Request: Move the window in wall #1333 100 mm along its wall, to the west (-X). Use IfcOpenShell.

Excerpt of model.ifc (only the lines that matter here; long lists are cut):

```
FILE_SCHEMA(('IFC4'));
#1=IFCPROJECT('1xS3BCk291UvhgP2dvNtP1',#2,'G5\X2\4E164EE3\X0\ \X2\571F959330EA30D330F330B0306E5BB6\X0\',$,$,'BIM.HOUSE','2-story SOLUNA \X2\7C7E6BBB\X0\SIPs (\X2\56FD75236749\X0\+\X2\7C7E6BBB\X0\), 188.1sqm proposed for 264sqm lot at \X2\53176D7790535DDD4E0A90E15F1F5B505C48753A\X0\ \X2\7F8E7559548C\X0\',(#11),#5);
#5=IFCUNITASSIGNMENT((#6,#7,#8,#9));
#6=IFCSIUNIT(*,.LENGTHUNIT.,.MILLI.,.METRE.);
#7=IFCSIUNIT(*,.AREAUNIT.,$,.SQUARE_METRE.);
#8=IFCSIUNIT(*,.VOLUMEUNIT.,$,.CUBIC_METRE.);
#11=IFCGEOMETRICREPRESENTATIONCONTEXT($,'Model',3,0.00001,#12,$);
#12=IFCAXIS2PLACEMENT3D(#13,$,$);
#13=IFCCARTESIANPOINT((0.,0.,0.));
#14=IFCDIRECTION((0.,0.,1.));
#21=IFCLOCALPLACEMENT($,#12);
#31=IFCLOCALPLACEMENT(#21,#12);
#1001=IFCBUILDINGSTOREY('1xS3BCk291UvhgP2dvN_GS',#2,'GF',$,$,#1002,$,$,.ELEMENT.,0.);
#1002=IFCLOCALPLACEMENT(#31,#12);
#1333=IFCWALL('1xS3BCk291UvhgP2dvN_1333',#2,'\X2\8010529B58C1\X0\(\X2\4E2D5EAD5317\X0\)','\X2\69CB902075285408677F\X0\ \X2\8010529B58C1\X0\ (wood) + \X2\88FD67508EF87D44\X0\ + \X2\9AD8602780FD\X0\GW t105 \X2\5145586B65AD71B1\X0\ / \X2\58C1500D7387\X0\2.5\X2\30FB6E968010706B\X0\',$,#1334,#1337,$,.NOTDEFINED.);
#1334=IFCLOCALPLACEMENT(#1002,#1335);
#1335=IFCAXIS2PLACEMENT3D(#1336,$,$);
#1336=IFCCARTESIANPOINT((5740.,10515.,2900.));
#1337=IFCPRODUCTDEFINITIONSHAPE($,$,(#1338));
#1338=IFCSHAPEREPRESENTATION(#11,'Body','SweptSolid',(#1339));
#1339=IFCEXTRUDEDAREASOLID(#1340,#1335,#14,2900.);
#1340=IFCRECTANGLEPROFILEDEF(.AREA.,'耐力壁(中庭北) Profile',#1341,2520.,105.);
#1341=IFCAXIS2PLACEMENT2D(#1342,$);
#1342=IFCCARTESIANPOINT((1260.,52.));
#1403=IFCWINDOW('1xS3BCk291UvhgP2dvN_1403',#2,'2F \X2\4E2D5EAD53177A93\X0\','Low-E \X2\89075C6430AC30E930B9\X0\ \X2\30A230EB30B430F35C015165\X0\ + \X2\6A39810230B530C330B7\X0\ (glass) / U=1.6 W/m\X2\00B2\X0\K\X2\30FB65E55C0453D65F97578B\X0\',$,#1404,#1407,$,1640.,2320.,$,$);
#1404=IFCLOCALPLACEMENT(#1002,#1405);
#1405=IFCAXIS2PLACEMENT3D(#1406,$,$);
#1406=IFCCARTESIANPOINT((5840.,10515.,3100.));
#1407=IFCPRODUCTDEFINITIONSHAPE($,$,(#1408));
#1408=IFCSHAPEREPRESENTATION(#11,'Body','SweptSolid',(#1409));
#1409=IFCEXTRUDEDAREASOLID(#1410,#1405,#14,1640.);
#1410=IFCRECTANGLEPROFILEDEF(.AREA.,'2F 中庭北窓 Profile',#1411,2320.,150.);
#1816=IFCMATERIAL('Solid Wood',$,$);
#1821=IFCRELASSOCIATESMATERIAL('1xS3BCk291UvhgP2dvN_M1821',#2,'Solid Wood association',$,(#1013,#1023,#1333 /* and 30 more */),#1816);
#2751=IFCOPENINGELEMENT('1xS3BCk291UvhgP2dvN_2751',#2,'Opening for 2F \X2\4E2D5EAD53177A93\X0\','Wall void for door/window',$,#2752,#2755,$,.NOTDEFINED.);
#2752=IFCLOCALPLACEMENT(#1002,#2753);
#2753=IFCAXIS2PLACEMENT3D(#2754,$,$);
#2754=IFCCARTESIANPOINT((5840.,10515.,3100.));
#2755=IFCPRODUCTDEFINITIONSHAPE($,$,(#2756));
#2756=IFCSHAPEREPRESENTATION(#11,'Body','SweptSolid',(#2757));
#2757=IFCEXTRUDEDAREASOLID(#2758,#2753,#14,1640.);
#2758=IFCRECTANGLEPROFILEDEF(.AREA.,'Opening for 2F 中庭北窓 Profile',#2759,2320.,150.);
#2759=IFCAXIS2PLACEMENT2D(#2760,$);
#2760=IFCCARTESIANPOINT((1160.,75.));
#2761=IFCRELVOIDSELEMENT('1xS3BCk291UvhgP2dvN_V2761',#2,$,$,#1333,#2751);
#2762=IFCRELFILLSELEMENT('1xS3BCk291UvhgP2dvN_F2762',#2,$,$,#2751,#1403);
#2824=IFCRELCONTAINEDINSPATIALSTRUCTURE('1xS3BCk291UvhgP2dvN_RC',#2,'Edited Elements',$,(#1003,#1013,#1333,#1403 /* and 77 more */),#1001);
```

```python
import ifcopenshell
import ifcopenshell.api.geometry
import ifcopenshell.util.placement
import ifcopenshell.util.unit

model = ifcopenshell.open("model.ifc")
unit_scale = ifcopenshell.util.unit.calculate_unit_scale(model)

window = model.by_guid("1xS3BCk291UvhgP2dvN_1403")
opening = window.FillsVoids[0].RelatingOpeningElement
wall = opening.VoidsElements[0].RelatingBuildingElement

wall_matrix = ifcopenshell.util.placement.get_local_placement(wall.ObjectPlacement)
shift = wall_matrix[:3, 0] * -0.1 / unit_scale
before = ifcopenshell.util.placement.get_local_placement(window.ObjectPlacement)[:3, 3].copy()

# The window is not placed relative to its opening, so move both.
for product in (opening, window):
    matrix = ifcopenshell.util.placement.get_local_placement(product.ObjectPlacement)
    matrix[:3, 3] += shift
    ifcopenshell.api.geometry.edit_object_placement(model, product=product, matrix=matrix, is_si=False)

after = ifcopenshell.util.placement.get_local_placement(window.ObjectPlacement)[:3, 3]
print("window moved by", (after - before).round(3) + 0.0)

model.write("model_v2.ifc")
```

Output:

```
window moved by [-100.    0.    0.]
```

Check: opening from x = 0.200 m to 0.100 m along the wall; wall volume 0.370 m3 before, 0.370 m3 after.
